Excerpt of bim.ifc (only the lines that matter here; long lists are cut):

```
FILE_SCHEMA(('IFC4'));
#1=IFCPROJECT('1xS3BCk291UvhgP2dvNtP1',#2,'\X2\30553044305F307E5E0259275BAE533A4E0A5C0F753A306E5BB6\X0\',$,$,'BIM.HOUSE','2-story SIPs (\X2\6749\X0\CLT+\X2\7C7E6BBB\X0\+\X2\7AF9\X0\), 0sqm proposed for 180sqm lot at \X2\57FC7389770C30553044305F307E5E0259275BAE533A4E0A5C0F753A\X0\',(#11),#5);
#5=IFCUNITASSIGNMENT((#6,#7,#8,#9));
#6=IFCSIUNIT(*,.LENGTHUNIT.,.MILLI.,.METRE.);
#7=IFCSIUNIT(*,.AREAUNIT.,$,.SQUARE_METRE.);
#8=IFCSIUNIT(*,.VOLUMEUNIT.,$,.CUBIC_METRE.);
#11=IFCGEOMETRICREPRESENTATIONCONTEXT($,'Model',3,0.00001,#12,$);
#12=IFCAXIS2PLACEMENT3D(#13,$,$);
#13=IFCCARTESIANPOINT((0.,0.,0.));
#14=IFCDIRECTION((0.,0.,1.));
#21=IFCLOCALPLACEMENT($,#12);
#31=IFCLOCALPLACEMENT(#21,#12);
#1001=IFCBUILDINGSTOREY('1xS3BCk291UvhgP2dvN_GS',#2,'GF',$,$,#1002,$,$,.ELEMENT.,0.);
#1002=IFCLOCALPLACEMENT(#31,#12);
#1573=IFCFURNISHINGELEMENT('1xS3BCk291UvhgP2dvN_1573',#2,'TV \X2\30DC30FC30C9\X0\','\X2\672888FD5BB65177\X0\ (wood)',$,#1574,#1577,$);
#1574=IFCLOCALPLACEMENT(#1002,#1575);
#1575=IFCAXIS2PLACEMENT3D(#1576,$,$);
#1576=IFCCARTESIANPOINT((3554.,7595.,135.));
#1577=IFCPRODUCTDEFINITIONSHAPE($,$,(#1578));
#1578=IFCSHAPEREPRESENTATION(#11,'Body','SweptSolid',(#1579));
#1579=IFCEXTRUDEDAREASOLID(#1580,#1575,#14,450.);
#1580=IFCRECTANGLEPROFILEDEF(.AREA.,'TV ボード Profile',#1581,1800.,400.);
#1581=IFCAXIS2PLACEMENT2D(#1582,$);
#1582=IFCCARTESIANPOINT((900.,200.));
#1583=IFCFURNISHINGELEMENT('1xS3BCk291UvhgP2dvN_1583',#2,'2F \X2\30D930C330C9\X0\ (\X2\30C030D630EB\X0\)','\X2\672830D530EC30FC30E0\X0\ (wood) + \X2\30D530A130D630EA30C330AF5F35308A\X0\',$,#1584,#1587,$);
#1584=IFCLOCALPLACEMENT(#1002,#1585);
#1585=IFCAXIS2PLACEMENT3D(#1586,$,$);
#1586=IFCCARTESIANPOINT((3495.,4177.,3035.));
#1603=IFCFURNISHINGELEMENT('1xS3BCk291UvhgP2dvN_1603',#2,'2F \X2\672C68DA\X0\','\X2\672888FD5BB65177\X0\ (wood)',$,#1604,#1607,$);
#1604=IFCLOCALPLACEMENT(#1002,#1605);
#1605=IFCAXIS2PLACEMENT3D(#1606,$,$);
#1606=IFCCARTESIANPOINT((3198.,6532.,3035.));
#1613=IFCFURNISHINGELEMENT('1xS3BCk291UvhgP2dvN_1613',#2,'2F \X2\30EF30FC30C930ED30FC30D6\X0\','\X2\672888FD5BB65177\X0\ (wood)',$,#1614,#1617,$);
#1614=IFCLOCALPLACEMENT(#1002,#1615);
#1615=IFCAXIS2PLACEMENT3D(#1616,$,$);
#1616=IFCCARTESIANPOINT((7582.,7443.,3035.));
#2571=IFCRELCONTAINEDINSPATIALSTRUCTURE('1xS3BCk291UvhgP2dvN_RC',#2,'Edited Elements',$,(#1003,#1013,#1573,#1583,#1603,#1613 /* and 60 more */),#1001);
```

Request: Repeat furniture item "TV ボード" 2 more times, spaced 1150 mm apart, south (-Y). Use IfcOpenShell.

```python
import numpy as np
import ifcopenshell
import ifcopenshell.api.geometry
import ifcopenshell.api.root
import ifcopenshell.util.element
import ifcopenshell.util.placement

model = ifcopenshell.open("bim.ifc")


def reuse_history(source, copy):
    """copy_class also copies each property set's owner history, people and application; keep the originals."""
    for rel in copy.IsDefinedBy:
        if rel.is_a("IfcRelDefinesByProperties") and (history := rel.RelatingPropertyDefinition.OwnerHistory):
            rel.RelatingPropertyDefinition.OwnerHistory = source.OwnerHistory
            ifcopenshell.util.element.remove_deep2(model, history)


source = model.by_guid("1xS3BCk291UvhgP2dvN_1573")
base = ifcopenshell.util.placement.get_local_placement(source.ObjectPlacement)
step = np.array([0.0, -1.0, 0.0]) * 1150.0

for i in range(1, 3):
    copy = ifcopenshell.api.root.copy_class(model, product=source)
    copy.Representation = ifcopenshell.util.element.copy_deep(
        model, source.Representation, exclude=["IfcGeometricRepresentationContext", "IfcRepresentationMap"]
    )
    reuse_history(source, copy)
    matrix = base.copy()
    matrix[:3, 3] += i * step
    print("added at", matrix[:3, 3].round(3) + 0.0)
    ifcopenshell.api.geometry.edit_object_placement(model, product=copy, matrix=matrix, is_si=False)

model.write("bim_updated.ifc")
```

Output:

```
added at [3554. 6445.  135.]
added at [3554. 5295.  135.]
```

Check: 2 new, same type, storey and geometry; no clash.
